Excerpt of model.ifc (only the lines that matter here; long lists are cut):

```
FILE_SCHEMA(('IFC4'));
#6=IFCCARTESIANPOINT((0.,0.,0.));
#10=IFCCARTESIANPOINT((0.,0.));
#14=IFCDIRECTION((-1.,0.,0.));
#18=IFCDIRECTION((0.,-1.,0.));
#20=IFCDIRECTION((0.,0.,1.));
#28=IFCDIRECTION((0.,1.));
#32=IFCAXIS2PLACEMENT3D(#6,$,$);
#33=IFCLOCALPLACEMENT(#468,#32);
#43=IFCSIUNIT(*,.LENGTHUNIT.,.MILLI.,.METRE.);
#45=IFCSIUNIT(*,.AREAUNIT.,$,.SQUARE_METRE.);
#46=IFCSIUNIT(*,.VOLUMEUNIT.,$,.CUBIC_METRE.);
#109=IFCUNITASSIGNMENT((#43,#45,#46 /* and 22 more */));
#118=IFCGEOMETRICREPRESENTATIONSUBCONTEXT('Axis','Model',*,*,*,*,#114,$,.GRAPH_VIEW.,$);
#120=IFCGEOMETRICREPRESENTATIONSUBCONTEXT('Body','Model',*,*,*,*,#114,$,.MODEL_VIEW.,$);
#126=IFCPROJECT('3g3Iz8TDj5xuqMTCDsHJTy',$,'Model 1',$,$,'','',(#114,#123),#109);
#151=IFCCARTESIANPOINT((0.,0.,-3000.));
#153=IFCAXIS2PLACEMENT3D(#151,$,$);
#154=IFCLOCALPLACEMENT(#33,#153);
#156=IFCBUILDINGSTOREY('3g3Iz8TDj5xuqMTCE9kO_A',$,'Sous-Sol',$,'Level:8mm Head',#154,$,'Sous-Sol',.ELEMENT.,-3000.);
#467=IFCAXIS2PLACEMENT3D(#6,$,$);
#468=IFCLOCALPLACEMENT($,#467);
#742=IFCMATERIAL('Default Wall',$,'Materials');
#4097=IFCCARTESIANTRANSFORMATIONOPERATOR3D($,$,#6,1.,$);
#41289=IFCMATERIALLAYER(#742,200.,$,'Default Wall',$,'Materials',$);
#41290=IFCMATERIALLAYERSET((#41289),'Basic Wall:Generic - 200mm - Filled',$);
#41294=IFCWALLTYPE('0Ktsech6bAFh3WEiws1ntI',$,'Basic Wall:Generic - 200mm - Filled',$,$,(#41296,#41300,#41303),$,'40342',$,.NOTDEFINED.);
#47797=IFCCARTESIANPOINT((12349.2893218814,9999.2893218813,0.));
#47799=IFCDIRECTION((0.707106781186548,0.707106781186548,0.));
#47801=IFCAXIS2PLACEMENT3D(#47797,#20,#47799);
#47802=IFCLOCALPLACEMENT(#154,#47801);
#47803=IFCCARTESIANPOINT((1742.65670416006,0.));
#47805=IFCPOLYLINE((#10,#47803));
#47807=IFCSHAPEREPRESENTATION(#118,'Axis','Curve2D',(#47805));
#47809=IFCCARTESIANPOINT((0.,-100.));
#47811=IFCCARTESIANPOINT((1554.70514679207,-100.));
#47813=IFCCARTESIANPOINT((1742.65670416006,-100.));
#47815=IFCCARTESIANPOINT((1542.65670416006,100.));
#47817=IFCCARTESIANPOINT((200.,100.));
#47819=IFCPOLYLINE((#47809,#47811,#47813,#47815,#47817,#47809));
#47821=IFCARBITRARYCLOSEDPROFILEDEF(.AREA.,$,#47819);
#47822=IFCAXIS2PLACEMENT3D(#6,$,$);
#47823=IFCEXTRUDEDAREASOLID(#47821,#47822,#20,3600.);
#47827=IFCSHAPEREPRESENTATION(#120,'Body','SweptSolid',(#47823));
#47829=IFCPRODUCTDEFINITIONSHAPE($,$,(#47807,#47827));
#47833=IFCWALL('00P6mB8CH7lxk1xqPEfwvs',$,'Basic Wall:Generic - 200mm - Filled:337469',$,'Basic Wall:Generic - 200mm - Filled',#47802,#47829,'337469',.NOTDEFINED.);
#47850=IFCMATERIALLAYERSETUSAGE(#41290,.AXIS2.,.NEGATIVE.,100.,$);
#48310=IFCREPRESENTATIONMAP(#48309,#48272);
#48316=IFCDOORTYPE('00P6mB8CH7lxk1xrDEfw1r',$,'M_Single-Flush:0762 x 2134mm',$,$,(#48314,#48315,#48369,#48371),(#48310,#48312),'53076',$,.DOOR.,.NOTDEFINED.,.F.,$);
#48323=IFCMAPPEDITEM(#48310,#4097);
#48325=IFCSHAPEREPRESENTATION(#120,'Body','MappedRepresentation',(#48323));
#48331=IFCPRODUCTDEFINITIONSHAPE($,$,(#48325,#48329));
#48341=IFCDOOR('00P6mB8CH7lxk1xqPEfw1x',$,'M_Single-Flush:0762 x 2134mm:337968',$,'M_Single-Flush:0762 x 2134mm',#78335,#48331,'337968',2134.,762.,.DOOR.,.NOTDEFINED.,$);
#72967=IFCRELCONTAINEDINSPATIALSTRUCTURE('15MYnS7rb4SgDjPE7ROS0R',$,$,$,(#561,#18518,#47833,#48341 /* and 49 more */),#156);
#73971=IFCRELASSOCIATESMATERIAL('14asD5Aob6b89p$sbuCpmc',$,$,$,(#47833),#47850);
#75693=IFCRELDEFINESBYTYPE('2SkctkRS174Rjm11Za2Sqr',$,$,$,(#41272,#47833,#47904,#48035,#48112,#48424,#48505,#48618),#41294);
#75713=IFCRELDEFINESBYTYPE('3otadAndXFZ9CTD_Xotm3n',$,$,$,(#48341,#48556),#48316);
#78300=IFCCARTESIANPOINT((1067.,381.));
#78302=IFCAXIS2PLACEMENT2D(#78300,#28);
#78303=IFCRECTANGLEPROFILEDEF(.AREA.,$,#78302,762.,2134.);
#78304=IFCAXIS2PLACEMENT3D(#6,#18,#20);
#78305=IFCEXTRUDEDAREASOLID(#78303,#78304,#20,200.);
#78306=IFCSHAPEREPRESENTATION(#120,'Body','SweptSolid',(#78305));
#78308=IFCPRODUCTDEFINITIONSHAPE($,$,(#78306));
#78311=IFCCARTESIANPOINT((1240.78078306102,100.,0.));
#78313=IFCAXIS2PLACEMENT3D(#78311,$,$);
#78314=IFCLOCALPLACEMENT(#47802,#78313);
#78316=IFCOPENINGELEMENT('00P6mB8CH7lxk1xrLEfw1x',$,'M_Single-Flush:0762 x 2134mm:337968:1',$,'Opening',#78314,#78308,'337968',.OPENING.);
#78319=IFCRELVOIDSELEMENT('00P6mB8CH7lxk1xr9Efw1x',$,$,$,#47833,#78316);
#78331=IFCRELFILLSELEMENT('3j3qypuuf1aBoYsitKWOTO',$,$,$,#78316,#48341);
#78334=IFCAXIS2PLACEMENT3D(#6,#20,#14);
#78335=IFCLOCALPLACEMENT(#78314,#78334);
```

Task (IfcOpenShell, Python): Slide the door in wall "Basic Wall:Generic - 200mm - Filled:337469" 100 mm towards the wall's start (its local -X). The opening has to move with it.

```python
import ifcopenshell
import ifcopenshell.api.geometry
import ifcopenshell.util.placement
import ifcopenshell.util.unit

model = ifcopenshell.open("model.ifc")
unit_scale = ifcopenshell.util.unit.calculate_unit_scale(model)

door = model.by_id(48341)
opening = door.FillsVoids[0].RelatingOpeningElement
wall = opening.VoidsElements[0].RelatingBuildingElement

wall_matrix = ifcopenshell.util.placement.get_local_placement(wall.ObjectPlacement)
shift = wall_matrix[:3, 0] * -0.1 / unit_scale
before = ifcopenshell.util.placement.get_local_placement(door.ObjectPlacement)[:3, 3].copy()

# The door is placed relative to its opening, so it follows when the opening moves.
matrix = ifcopenshell.util.placement.get_local_placement(opening.ObjectPlacement)
matrix[:3, 3] += shift
ifcopenshell.api.geometry.edit_object_placement(
    model, product=opening, matrix=matrix, is_si=False, should_transform_children=True
)

after = ifcopenshell.util.placement.get_local_placement(door.ObjectPlacement)[:3, 3]
print("door moved by", (after - before).round(3) + 0.0)

model.write("model-out.ifc")
```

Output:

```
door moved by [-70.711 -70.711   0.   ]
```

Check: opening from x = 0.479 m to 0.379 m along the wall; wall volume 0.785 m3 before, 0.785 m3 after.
